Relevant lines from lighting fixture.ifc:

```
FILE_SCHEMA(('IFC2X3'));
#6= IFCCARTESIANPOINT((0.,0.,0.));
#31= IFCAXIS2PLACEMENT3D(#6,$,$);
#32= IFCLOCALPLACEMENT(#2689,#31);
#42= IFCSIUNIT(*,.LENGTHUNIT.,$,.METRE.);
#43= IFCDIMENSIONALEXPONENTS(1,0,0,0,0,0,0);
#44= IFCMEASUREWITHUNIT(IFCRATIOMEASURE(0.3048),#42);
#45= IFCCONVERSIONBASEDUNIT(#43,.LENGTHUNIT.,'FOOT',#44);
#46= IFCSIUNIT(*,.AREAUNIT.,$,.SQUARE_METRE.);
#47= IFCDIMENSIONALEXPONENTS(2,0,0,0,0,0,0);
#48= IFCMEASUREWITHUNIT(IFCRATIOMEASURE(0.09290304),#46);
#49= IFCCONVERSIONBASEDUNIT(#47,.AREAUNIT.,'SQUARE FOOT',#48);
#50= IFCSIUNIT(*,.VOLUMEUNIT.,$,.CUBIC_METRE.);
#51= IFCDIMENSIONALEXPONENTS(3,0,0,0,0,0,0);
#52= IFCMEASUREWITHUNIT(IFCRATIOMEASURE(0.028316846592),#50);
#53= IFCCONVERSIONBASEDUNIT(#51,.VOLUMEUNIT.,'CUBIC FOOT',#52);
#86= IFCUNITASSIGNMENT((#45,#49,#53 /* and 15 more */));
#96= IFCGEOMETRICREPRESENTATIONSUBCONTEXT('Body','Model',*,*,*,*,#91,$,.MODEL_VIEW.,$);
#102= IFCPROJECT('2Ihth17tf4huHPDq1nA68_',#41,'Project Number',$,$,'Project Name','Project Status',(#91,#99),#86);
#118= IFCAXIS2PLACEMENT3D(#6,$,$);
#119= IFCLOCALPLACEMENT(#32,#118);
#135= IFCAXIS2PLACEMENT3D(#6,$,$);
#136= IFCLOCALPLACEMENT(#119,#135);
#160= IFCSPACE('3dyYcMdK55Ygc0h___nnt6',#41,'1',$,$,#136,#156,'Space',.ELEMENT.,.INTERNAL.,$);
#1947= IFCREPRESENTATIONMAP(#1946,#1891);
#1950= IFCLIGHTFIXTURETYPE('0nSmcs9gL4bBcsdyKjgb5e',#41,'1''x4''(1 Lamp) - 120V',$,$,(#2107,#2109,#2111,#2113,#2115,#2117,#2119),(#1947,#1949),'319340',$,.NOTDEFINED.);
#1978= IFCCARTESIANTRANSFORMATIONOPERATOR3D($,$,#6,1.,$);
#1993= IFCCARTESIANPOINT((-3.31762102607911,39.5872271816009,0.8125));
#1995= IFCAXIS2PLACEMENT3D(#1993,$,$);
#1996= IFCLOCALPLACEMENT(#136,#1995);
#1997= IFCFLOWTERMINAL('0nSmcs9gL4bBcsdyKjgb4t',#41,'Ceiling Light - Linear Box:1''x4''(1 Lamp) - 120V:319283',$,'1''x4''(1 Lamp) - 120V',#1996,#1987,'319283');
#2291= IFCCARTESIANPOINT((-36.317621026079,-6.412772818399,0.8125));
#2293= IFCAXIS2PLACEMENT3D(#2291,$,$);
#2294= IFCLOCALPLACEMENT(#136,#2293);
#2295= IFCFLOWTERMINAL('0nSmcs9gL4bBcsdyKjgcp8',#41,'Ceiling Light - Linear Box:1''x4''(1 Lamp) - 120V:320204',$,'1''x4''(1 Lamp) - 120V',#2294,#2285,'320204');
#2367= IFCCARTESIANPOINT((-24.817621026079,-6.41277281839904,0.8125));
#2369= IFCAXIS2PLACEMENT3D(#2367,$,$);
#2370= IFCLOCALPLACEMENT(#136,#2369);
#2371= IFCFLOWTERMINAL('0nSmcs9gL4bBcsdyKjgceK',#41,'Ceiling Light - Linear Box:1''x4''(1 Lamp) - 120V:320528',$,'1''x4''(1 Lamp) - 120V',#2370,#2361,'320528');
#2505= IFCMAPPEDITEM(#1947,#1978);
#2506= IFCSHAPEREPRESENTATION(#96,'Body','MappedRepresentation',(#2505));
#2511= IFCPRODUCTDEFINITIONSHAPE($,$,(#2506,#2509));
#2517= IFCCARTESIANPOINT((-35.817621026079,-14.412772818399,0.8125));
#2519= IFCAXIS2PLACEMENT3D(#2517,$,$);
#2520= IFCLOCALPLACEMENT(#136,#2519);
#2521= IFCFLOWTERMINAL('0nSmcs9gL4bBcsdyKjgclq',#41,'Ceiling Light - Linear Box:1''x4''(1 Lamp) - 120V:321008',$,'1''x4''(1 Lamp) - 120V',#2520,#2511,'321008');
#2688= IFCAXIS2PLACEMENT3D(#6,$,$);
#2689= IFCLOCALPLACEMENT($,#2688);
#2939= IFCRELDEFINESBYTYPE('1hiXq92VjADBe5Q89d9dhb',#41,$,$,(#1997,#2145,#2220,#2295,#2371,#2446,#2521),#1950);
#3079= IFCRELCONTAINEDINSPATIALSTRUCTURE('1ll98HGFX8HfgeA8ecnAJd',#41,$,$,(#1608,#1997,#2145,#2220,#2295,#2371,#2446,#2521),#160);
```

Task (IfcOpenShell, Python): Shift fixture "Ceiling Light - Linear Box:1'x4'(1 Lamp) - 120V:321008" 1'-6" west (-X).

```python
import ifcopenshell
import ifcopenshell.api.geometry
import ifcopenshell.util.placement
import ifcopenshell.util.unit

model = ifcopenshell.open("lighting fixture.ifc")
unit_scale = ifcopenshell.util.unit.calculate_unit_scale(model)

item = model.by_guid("0nSmcs9gL4bBcsdyKjgclq")
matrix = ifcopenshell.util.placement.get_local_placement(item.ObjectPlacement)
matrix[0, 3] -= 18 * 0.0254 / unit_scale
ifcopenshell.api.geometry.edit_object_placement(model, product=item, matrix=matrix, is_si=False)

print(ifcopenshell.util.placement.get_local_placement(item.ObjectPlacement).round(3) + 0.0)

model.write("lighting fixture_rev.ifc")
```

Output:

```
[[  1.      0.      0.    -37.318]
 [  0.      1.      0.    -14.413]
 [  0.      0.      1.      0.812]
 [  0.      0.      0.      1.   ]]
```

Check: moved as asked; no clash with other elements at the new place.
